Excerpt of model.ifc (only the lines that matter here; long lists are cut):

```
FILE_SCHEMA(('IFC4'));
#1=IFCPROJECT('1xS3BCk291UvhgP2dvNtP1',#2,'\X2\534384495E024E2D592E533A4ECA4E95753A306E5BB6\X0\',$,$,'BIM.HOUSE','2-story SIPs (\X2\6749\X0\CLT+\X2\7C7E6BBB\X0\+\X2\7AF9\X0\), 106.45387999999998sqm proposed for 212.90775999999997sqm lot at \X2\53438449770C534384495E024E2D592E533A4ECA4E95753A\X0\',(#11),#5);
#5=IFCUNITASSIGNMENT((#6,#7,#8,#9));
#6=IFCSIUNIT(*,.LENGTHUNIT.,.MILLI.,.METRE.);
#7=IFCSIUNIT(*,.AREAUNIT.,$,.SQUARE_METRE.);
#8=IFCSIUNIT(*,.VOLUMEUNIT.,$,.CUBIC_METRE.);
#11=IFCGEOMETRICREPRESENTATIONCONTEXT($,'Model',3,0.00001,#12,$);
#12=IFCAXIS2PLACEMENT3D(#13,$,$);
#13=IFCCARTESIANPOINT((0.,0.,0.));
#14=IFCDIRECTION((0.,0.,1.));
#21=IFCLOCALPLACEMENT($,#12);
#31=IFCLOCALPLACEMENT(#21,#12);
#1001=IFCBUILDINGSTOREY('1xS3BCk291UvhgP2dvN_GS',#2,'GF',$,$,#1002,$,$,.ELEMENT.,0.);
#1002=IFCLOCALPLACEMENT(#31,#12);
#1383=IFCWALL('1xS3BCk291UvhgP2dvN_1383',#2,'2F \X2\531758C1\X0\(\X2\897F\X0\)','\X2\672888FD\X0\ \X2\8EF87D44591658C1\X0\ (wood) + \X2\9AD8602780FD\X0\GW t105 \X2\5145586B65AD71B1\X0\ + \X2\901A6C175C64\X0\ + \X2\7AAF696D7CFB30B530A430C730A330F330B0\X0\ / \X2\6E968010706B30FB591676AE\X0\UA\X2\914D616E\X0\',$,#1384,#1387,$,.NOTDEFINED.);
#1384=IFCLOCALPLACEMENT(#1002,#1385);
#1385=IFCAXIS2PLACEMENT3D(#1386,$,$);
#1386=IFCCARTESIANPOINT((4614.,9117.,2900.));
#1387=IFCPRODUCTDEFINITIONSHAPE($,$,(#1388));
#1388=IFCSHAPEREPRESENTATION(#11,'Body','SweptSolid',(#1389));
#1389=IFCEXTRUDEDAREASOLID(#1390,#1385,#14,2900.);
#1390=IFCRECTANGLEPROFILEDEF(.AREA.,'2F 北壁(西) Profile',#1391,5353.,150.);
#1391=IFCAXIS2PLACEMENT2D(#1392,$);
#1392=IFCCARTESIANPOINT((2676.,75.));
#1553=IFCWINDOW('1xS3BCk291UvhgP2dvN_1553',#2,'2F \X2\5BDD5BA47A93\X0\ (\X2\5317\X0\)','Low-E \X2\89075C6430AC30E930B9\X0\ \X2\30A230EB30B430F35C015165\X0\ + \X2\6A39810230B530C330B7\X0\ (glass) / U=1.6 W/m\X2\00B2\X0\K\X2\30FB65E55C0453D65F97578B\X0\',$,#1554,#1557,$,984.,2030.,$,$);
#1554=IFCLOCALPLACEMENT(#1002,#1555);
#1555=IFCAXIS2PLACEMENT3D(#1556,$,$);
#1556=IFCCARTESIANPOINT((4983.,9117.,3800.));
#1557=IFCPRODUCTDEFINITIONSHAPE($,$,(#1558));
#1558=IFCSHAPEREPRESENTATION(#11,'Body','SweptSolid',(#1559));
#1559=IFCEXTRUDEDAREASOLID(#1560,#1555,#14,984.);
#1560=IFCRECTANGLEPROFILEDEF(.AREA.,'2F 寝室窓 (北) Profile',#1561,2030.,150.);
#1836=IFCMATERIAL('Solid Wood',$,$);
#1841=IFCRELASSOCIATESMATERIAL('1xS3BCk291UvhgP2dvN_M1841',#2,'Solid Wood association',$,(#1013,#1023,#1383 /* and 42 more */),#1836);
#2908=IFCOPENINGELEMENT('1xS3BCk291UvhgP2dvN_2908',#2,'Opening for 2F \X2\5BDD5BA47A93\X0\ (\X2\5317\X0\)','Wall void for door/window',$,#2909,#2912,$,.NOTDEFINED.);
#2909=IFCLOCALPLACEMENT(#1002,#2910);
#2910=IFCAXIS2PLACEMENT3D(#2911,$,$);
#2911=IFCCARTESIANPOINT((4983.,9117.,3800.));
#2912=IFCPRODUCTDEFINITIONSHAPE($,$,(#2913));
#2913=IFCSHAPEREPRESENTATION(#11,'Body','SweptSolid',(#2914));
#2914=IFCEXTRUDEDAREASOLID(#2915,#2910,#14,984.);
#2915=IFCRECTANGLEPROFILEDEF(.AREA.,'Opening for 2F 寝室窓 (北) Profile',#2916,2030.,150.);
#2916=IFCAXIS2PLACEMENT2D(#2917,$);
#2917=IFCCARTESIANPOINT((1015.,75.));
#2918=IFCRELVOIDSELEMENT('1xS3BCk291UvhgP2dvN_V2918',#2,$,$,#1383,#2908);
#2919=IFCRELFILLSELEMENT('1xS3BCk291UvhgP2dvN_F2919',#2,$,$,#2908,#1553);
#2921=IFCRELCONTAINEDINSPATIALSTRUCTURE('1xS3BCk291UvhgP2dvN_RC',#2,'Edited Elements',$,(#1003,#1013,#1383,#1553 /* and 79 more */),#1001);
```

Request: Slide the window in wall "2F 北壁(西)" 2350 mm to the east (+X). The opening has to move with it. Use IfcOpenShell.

```python
import ifcopenshell
import ifcopenshell.api.geometry
import ifcopenshell.util.placement
import ifcopenshell.util.unit

model = ifcopenshell.open("model.ifc")
unit_scale = ifcopenshell.util.unit.calculate_unit_scale(model)

window = model.by_id(1553)
opening = window.FillsVoids[0].RelatingOpeningElement
wall = opening.VoidsElements[0].RelatingBuildingElement

wall_matrix = ifcopenshell.util.placement.get_local_placement(wall.ObjectPlacement)
shift = wall_matrix[:3, 0] * 2.35 / unit_scale
before = ifcopenshell.util.placement.get_local_placement(window.ObjectPlacement)[:3, 3].copy()

# The window is not placed relative to its opening, so move both.
for product in (opening, window):
    matrix = ifcopenshell.util.placement.get_local_placement(product.ObjectPlacement)
    matrix[:3, 3] += shift
    ifcopenshell.api.geometry.edit_object_placement(model, product=product, matrix=matrix, is_si=False)

after = ifcopenshell.util.placement.get_local_placement(window.ObjectPlacement)[:3, 3]
print("window moved by", (after - before).round(3) + 0.0)

model.write("model_v2.ifc")
```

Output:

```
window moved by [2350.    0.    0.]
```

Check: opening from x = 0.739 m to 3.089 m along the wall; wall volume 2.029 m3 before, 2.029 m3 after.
